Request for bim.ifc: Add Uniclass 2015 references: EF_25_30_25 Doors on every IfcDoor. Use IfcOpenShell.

First a look at what the model holds.

```python
import ifcopenshell

model = ifcopenshell.open("bim.ifc")
print(model.schema)
print("classifications:", [c.Name for c in model.by_type("IfcClassification")])
for ifc_class in ("IfcDoor", "IfcRoof", "IfcStair", "IfcWall", "IfcWindow"):
    print(ifc_class, len(model.by_type(ifc_class)))
```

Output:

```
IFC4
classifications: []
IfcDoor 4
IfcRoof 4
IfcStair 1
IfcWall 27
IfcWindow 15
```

```python
import ifcopenshell
import ifcopenshell.api.classification

model = ifcopenshell.open("bim.ifc")

system = ifcopenshell.api.classification.add_classification(model, classification="Uniclass 2015")

codes = {
    "IfcDoor": ("EF_25_30_25", "Doors"),
}
for ifc_class, (code, name) in codes.items():
    products = model.by_type(ifc_class)
    ifcopenshell.api.classification.add_reference(
        model, products=products, classification=system, identification=code, name=name
    )
    print(code, len(products))

model.write("bim_rev.ifc")
```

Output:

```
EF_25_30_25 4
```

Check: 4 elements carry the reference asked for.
